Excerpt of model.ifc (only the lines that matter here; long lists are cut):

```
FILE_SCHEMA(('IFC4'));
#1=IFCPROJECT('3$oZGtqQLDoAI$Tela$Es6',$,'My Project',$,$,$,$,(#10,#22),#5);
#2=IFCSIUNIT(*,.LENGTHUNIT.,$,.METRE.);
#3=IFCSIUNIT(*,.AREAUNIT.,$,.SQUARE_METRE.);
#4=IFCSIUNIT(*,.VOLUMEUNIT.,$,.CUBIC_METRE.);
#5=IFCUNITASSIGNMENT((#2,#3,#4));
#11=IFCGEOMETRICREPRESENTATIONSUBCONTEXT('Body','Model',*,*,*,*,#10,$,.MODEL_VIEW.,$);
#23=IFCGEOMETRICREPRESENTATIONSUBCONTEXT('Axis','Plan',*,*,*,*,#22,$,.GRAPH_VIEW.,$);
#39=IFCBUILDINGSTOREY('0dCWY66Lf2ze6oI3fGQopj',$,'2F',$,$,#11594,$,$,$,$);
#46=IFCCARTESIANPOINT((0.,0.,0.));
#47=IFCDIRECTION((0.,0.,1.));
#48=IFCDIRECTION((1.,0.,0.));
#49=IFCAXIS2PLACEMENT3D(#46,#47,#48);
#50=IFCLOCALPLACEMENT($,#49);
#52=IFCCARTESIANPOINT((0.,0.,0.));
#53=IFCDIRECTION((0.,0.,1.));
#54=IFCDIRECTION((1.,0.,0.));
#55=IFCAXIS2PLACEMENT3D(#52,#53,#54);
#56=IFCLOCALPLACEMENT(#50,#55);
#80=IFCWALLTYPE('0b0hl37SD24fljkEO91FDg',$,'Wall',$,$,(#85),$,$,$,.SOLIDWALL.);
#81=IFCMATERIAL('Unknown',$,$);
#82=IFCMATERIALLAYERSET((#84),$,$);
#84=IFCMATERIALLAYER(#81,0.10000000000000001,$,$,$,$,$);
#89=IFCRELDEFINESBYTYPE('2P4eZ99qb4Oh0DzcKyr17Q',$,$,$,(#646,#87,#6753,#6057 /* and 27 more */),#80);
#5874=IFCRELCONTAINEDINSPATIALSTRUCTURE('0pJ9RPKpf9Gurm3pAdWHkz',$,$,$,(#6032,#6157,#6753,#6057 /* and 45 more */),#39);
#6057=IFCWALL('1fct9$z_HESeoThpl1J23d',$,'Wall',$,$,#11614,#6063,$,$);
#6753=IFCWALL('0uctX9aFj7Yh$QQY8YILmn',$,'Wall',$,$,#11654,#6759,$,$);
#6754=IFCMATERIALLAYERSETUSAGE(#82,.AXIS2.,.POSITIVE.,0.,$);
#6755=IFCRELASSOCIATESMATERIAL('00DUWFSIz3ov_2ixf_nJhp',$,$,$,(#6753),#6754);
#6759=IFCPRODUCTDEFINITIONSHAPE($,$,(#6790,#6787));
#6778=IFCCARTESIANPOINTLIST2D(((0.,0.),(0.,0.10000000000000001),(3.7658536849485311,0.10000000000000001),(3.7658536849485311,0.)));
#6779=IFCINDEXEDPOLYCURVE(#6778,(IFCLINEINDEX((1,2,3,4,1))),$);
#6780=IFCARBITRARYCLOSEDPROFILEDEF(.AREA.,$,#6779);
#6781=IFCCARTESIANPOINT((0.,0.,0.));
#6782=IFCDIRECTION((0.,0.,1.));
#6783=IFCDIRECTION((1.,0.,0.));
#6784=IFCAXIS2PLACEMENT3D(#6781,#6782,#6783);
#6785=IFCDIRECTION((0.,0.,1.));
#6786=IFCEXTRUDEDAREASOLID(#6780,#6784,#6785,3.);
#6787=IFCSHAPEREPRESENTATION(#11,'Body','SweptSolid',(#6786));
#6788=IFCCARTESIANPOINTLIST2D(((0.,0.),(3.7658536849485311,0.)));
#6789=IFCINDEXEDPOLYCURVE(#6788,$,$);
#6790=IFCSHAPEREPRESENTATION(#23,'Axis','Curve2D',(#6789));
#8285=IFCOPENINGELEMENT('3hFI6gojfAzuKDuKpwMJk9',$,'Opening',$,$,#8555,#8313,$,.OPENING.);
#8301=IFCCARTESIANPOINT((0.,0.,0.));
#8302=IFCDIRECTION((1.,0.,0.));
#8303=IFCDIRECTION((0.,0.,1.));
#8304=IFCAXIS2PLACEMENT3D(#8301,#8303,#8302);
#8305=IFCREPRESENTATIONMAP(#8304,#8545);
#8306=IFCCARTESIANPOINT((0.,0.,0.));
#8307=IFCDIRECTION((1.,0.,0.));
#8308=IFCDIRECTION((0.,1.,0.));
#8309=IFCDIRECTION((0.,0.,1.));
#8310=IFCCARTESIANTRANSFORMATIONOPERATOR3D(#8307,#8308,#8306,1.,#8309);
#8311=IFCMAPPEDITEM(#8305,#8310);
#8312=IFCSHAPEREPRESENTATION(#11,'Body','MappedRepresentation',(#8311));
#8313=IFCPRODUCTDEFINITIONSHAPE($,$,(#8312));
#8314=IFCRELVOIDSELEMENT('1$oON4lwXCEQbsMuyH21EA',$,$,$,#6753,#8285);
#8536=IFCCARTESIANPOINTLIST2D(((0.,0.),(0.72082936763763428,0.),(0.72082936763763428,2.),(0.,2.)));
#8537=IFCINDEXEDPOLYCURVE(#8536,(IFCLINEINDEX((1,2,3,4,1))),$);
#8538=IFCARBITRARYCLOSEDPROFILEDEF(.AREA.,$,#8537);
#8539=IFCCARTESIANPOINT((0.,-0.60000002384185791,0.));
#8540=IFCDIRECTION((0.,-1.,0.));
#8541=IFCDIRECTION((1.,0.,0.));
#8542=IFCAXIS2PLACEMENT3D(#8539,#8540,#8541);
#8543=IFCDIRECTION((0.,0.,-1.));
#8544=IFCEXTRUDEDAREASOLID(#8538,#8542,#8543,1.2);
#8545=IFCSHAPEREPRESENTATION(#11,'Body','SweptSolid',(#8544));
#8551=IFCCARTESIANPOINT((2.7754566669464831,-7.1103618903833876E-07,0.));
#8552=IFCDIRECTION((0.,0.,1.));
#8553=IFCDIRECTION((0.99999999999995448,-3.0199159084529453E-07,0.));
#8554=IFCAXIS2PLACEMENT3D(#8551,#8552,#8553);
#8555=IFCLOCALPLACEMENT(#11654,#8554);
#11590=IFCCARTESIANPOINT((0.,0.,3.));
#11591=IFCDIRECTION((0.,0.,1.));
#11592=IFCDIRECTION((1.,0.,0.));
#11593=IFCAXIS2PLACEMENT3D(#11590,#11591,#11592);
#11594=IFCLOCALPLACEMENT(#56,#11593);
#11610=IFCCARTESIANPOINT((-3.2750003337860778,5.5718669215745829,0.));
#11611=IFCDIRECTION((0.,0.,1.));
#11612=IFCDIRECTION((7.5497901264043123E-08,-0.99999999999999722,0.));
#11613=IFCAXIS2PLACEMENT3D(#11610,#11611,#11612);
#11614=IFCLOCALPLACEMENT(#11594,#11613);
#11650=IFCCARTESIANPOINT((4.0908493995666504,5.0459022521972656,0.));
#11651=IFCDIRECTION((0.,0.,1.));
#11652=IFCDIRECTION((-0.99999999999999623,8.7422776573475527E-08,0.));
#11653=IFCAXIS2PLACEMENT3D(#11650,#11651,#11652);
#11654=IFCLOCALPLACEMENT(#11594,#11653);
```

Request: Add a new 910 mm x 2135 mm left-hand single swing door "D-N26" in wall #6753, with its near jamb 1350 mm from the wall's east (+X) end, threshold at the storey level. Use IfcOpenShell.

```python
import numpy as np
import ifcopenshell
import ifcopenshell.api.feature
import ifcopenshell.api.geometry
import ifcopenshell.api.root
import ifcopenshell.api.spatial
import ifcopenshell.geom
import ifcopenshell.util.element
import ifcopenshell.util.placement
import ifcopenshell.util.representation
import ifcopenshell.util.shape
import ifcopenshell.util.unit

model = ifcopenshell.open("model.ifc")
unit_scale = ifcopenshell.util.unit.calculate_unit_scale(model)
settings = ifcopenshell.geom.settings()


def volume(element):
    """Net volume in cubic metres, openings subtracted."""
    shape = ifcopenshell.geom.create_shape(settings, element)
    return ifcopenshell.util.shape.get_volume(shape.geometry)


wall = model.by_id(6753)
storey = ifcopenshell.util.element.get_container(wall, ifc_class="IfcBuildingStorey")
context = ifcopenshell.util.representation.get_context(model, "Model", "Body", "MODEL_VIEW")
before = volume(wall)

width, height, from_end, sill = 0.91, 2.135, 1.35, 0.0  # metres

# The wall runs along its own X axis, and the end named is its -X end.
wall_shape = ifcopenshell.geom.create_shape(settings, wall)
x, y, z = ifcopenshell.util.shape.get_vertices(wall_shape.geometry).T
start = x.min() + from_end
face, thickness = float(y.min()), float(y.max() - y.min())
wall_matrix = ifcopenshell.util.placement.get_local_placement(wall.ObjectPlacement)
level = ifcopenshell.util.placement.get_local_placement(storey.ObjectPlacement)[2, 3]


def in_wall(x, y):
    """Placement at x, y metres in the wall's axes, at sill height."""
    matrix = wall_matrix.copy()
    matrix[:, 3] = wall_matrix @ np.array([x / unit_scale, y / unit_scale, 0.0, 1.0])
    matrix[2, 3] = level + sill / unit_scale
    return matrix


# Opening: a box that overshoots both wall faces by 50 mm.
opening = ifcopenshell.api.root.create_entity(model, ifc_class="IfcOpeningElement", predefined_type="OPENING")
box = ifcopenshell.api.geometry.add_wall_representation(
    model, context=context, length=width, height=height, thickness=thickness + 0.1
)
ifcopenshell.api.geometry.assign_representation(model, product=opening, representation=box)
ifcopenshell.api.geometry.edit_object_placement(model, product=opening, matrix=in_wall(start, face - 0.05), is_si=False)
ifcopenshell.api.feature.add_feature(model, feature=opening, element=wall)

door = ifcopenshell.api.root.create_entity(model, ifc_class="IfcDoor", name="D-N26", predefined_type="DOOR")
door.OverallWidth, door.OverallHeight = width / unit_scale, height / unit_scale
door.OperationType = "SINGLE_SWING_LEFT"
body = ifcopenshell.api.geometry.add_door_representation(
    model,
    context=context,
    overall_width=door.OverallWidth,
    overall_height=door.OverallHeight,
    operation_type="SINGLE_SWING_LEFT",
    lining_properties={"LiningDepth": thickness / unit_scale, "ThresholdDepth": thickness / unit_scale},
)
ifcopenshell.api.geometry.assign_representation(model, product=door, representation=body)
ifcopenshell.api.spatial.assign_container(model, products=[door], relating_structure=storey)
ifcopenshell.api.feature.add_filling(model, opening=opening, element=door)

# The lining spans the wall, so the door starts at the wall face.
ifcopenshell.api.geometry.edit_object_placement(model, product=door, matrix=in_wall(start, face), is_si=False)

after = volume(wall)

print(f"wall volume {before:.3f} -> {after:.3f} m3")

model.write("model_rev.ifc")
```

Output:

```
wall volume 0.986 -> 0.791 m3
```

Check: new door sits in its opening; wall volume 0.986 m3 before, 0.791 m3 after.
